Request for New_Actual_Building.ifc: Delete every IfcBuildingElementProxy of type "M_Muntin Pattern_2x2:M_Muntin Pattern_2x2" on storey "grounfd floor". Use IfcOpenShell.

First a look at what the model holds.

```python
import ifcopenshell
import ifcopenshell.util.element

model = ifcopenshell.open("New_Actual_Building.ifc")
print(model.schema)
storey = next(s for s in model.by_type("IfcBuildingStorey") if s.Name == "grounfd floor")
proxies = [e for e in ifcopenshell.util.element.get_decomposition(storey) if e.is_a("IfcBuildingElementProxy")]
seen = {}
for e in proxies:
    element_type = ifcopenshell.util.element.get_type(e)
    name = element_type.Name if element_type not in (None, e) else None
    seen[name] = seen.get(name, 0) + 1
for name, count in sorted(seen.items(), key=str):
    print(count, "x", name)
```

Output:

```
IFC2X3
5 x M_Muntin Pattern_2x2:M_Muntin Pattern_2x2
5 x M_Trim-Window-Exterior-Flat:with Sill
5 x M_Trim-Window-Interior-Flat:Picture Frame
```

```python
import ifcopenshell
import ifcopenshell.api.root
import ifcopenshell.util.element

model = ifcopenshell.open("New_Actual_Building.ifc")

storey = next(s for s in model.by_type("IfcBuildingStorey") if s.Name == "grounfd floor")
proxies = [e for e in ifcopenshell.util.element.get_decomposition(storey) if e.is_a("IfcBuildingElementProxy")]
targets = [e for e in proxies if (t := ifcopenshell.util.element.get_type(e)) not in (None, e) and t.Name == "M_Muntin Pattern_2x2:M_Muntin Pattern_2x2"]

for e in targets:
    ifcopenshell.api.root.remove_product(model, product=e)
print(len(targets), "removed")

model.write("New_Actual_Building_edited.ifc")
```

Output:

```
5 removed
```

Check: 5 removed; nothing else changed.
